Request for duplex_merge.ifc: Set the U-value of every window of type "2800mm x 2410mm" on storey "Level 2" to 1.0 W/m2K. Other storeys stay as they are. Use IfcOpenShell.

First a look at what the model holds.

```python
import ifcopenshell
import ifcopenshell.util.element

model = ifcopenshell.open("duplex_merge.ifc")
print(model.schema)
storey = next(s for s in model.by_type("IfcBuildingStorey") if s.Name == "Level 2")
windows = [e for e in ifcopenshell.util.element.get_decomposition(storey) if e.is_a("IfcWindow")]
seen = {}
for e in windows:
    element_type = ifcopenshell.util.element.get_type(e)
    key = (element_type.Name if element_type != e and element_type else None, ifcopenshell.util.element.get_pset(e, "Pset_WindowCommon", "ThermalTransmittance"))
    seen[key] = seen.get(key, 0) + 1
for (name, value), count in sorted(seen.items(), key=str):
    print(count, "x", name, "|", value)
```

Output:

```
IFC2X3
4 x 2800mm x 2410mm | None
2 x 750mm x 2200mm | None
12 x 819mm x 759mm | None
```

```python
import ifcopenshell
import ifcopenshell.api.pset
import ifcopenshell.util.element

model = ifcopenshell.open("duplex_merge.ifc")

storey = next(s for s in model.by_type("IfcBuildingStorey") if s.Name == "Level 2")
windows = [e for e in ifcopenshell.util.element.get_decomposition(storey) if e.is_a("IfcWindow")]

count = 0
for e in windows:
    element_type = ifcopenshell.util.element.get_type(e)
    if element_type in (None, e) or element_type.Name != "2800mm x 2410mm":
        continue
    # add_pset returns the element's existing set when there is one.
    pset = ifcopenshell.api.pset.add_pset(model, product=e, name="Pset_WindowCommon")
    ifcopenshell.api.pset.edit_pset(model, pset=pset, properties={"ThermalTransmittance": 1.0})
    count += 1

print(count, "windows updated")

model.write("duplex_merge_edited.ifc")
```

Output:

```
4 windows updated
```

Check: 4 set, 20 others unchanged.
